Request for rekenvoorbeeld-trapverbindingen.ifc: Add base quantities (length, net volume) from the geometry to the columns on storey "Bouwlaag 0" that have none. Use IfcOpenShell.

First a look at what the model holds.

```python
import ifcopenshell
import ifcopenshell.util.element
import ifcopenshell.util.unit

model = ifcopenshell.open("rekenvoorbeeld-trapverbindingen.ifc")
print(model.schema)
for unit_type in ("LENGTHUNIT", "AREAUNIT", "VOLUMEUNIT"):
    print(unit_type, ifcopenshell.util.unit.calculate_unit_scale(model, unit_type))
storey = next(s for s in model.by_type("IfcBuildingStorey") if s.Name == "Bouwlaag 0")
columns = [e for e in ifcopenshell.util.element.get_decomposition(storey) if e.is_a("IfcColumn")]
for e in sorted(columns, key=lambda e: e.id()):
    print(e.id(), e.is_a(), e.Name, list(ifcopenshell.util.element.get_psets(e, qtos_only=True)), sep=" | ")
```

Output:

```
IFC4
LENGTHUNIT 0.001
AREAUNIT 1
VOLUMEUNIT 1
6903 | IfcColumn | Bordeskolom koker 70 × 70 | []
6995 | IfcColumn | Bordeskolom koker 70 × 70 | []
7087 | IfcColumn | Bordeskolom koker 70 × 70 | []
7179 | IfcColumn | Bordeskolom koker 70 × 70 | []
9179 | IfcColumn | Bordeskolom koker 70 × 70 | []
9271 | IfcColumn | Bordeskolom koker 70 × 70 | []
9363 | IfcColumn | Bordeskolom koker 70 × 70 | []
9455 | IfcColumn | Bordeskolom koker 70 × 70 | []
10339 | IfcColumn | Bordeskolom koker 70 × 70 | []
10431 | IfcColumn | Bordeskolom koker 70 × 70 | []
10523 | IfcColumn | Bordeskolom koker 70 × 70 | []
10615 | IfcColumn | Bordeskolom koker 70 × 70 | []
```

```python
import ifcopenshell
import ifcopenshell.api.pset
import ifcopenshell.geom
import ifcopenshell.util.element
import ifcopenshell.util.shape
import ifcopenshell.util.unit

model = ifcopenshell.open("rekenvoorbeeld-trapverbindingen.ifc")
unit_scale = ifcopenshell.util.unit.calculate_unit_scale(model)
volume_scale = ifcopenshell.util.unit.calculate_unit_scale(model, "VOLUMEUNIT")
settings = ifcopenshell.geom.settings()

storey = next(s for s in model.by_type("IfcBuildingStorey") if s.Name == "Bouwlaag 0")
columns = [e for e in ifcopenshell.util.element.get_decomposition(storey) if e.is_a("IfcColumn")]

for e in sorted(columns, key=lambda e: e.id()):
    if ifcopenshell.util.element.get_psets(e, qtos_only=True, should_inherit=False):
        continue
    # Geometry comes back in metres, in the element's own axes.
    shape = ifcopenshell.geom.create_shape(settings, e)
    values = {
        "Length": ifcopenshell.util.shape.get_z(shape.geometry) / unit_scale,
        "NetVolume": ifcopenshell.util.shape.get_volume(shape.geometry) / volume_scale,
    }
    qto = ifcopenshell.api.pset.add_qto(model, product=e, name="Qto_ColumnBaseQuantities")
    ifcopenshell.api.pset.edit_qto(model, qto=qto, properties=values)
    print(e.id(), {k: round(v, 3) for k, v in values.items()})

model.write("rekenvoorbeeld-trapverbindingen_updated.ifc")
```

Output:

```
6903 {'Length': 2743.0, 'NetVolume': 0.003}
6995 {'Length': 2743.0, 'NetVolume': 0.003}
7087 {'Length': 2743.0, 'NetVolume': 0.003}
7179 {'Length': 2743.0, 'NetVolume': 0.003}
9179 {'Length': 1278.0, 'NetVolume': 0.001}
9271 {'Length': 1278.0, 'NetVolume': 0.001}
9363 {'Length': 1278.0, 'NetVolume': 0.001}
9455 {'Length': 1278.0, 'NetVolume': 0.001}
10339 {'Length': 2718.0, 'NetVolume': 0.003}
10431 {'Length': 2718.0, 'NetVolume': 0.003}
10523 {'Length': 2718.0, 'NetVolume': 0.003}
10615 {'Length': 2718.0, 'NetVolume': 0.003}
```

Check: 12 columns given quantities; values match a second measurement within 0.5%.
